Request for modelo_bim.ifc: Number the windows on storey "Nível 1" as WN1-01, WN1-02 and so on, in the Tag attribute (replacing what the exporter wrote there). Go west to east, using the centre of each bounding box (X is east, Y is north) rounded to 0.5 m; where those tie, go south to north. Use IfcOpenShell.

First a look at what the model holds.

```python
import ifcopenshell
import ifcopenshell.util.element
import ifcopenshell.util.placement

model = ifcopenshell.open("modelo_bim.ifc")
print(model.schema)
storey = next(s for s in model.by_type("IfcBuildingStorey") if s.Name == "Nível 1")
windows = [e for e in ifcopenshell.util.element.get_decomposition(storey) if e.is_a("IfcWindow")]
for e in sorted(windows, key=lambda e: e.id()):
    origin = ifcopenshell.util.placement.get_local_placement(e.ObjectPlacement)[:3, 3]
    print(e.id(), e.Tag, e.Name, origin.round(2) + 0.0, sep=" | ")
```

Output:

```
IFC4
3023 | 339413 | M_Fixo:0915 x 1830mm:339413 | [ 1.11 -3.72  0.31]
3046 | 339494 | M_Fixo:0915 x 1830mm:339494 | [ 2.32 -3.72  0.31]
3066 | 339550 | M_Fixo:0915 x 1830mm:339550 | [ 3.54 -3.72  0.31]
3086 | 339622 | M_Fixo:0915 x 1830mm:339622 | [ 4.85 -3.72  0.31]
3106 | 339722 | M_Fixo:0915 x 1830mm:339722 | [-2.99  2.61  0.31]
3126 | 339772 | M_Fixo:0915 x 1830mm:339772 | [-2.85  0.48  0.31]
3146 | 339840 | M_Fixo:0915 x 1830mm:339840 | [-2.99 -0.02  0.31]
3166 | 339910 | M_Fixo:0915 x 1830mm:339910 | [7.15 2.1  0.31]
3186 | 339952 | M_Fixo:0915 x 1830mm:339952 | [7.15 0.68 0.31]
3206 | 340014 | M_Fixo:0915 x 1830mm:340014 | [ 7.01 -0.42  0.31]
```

```python
import ifcopenshell
import ifcopenshell.geom
import ifcopenshell.util.element
import ifcopenshell.util.shape

model = ifcopenshell.open("modelo_bim.ifc")
settings = ifcopenshell.geom.settings()
settings.set("use-world-coords", True)


def centre(element):
    shape = ifcopenshell.geom.create_shape(settings, element)
    return ifcopenshell.util.shape.get_bbox_centroid(shape.geometry)


storey = next(s for s in model.by_type("IfcBuildingStorey") if s.Name == "Nível 1")
windows = [e for e in ifcopenshell.util.element.get_decomposition(storey) if e.is_a("IfcWindow")]

# Insertion points can sit at a corner or the storey origin, so sort by the geometry (in metres).
centres = {e: centre(e) for e in windows}
windows.sort(key=lambda e: (round(centres[e][0] / 0.5), centres[e][1]))

for i, e in enumerate(windows, start=1):
    number = f"WN1-{i:02d}"
    e.Tag = number
    print(e.id(), number)

model.write("modelo_bim_rev.ifc")
```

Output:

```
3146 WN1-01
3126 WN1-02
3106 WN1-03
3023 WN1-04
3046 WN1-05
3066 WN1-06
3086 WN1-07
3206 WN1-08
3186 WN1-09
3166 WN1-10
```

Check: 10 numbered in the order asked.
